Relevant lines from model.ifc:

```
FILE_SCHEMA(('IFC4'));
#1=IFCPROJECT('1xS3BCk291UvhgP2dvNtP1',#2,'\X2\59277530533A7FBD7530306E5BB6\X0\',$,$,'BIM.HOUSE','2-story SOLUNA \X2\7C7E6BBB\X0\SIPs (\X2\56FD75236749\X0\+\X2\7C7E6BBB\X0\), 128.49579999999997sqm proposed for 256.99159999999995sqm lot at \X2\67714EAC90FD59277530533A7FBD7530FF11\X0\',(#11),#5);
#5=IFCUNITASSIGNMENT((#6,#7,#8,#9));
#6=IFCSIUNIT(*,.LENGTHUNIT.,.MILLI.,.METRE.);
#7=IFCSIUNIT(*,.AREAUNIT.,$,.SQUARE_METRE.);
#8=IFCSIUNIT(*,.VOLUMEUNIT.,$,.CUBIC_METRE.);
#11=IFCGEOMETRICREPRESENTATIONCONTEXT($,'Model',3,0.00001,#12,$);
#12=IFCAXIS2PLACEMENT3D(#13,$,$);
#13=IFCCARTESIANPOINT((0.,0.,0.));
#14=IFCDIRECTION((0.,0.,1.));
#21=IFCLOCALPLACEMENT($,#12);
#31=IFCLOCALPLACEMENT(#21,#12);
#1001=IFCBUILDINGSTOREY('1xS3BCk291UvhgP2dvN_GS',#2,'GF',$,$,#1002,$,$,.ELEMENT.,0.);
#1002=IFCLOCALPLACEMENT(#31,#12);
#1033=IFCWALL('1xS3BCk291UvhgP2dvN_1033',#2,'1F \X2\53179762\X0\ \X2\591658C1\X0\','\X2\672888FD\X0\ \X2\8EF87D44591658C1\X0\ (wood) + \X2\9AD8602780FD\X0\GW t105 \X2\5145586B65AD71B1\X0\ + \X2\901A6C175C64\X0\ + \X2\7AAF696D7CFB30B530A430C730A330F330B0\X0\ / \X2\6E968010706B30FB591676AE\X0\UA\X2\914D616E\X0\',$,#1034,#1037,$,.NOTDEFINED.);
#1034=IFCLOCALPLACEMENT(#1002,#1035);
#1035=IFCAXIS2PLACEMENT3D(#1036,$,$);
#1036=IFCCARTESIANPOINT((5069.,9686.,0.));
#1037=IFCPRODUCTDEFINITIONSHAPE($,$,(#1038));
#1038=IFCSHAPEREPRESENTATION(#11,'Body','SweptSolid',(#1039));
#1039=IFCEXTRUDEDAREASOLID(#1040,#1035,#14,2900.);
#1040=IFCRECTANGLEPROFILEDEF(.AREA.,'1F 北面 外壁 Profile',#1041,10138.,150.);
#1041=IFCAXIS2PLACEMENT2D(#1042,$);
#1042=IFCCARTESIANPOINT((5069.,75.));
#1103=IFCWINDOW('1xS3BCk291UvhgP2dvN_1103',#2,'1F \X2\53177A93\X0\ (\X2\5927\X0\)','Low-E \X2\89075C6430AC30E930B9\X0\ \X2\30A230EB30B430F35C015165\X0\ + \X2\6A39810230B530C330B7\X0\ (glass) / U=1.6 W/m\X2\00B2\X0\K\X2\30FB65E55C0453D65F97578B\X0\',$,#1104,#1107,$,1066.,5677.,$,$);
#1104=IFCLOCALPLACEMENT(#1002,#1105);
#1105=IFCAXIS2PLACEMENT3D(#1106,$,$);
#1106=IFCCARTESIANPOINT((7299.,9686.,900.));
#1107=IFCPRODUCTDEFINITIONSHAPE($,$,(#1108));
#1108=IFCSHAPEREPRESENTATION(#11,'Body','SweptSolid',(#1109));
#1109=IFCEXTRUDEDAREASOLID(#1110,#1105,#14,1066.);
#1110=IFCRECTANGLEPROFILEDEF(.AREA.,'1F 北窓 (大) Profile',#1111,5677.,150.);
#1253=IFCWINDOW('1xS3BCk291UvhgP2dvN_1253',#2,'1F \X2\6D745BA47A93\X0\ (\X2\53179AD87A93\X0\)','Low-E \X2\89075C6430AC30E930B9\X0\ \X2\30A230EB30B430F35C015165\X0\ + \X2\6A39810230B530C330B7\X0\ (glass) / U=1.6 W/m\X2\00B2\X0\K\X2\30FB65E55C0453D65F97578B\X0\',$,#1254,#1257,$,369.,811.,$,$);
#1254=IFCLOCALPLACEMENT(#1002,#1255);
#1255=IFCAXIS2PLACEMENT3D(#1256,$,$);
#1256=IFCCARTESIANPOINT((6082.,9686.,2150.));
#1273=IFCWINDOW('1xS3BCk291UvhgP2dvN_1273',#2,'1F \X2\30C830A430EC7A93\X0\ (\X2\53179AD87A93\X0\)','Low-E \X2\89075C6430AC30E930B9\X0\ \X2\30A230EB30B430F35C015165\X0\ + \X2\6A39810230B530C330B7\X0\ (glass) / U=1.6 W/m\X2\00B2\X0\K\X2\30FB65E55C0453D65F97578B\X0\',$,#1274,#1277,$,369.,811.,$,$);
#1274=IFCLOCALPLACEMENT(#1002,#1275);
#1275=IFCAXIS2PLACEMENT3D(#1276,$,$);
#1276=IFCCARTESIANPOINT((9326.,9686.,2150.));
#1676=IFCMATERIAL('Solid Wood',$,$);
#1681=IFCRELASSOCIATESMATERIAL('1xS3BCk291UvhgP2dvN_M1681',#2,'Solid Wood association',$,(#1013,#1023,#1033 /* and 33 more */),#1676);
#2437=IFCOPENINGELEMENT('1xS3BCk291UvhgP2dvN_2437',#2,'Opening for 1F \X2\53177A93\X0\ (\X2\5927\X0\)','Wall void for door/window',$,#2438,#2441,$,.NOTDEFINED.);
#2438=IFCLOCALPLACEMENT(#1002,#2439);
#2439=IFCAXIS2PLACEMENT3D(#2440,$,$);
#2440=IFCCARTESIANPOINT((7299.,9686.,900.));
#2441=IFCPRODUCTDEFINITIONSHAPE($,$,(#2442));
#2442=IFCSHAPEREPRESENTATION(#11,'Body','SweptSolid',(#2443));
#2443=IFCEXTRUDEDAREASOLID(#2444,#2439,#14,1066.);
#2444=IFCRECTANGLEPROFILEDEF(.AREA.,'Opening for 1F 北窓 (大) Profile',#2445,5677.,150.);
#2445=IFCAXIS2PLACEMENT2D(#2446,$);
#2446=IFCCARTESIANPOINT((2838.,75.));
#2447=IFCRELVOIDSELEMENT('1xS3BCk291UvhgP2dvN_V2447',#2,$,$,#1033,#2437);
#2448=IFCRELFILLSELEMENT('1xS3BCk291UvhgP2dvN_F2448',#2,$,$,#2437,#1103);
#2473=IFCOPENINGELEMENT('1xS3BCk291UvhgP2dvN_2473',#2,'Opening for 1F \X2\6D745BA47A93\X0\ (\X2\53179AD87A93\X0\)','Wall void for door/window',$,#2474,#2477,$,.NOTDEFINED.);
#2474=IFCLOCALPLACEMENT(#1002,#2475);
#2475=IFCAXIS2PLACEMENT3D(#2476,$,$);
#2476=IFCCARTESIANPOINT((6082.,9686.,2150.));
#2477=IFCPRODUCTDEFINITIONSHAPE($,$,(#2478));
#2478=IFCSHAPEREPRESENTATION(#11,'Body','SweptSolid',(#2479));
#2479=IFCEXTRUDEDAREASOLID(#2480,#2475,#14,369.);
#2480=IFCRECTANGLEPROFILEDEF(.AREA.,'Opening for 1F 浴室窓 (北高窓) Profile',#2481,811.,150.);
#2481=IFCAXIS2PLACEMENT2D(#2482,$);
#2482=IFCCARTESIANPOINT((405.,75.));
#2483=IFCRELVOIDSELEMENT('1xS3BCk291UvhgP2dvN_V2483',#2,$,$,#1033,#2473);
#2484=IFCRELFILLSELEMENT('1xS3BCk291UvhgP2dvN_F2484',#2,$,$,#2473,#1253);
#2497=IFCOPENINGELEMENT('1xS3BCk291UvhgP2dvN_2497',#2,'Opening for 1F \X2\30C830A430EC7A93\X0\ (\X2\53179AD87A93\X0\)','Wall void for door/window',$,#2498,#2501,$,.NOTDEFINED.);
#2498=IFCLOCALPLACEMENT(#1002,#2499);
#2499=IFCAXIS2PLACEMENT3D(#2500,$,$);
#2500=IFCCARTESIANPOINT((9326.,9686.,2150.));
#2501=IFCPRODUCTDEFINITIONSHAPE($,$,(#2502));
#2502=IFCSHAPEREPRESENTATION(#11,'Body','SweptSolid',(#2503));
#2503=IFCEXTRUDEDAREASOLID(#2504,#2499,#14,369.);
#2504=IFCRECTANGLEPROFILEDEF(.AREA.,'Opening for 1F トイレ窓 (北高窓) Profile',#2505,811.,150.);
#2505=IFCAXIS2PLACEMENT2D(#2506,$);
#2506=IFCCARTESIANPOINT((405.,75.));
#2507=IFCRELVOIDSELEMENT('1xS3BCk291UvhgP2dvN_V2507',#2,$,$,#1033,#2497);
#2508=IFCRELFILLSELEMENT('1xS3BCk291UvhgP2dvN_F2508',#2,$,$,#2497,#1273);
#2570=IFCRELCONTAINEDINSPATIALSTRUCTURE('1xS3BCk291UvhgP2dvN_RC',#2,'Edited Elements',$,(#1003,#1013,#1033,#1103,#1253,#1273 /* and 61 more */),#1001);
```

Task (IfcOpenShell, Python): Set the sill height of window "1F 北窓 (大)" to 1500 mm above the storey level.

```python
import numpy as np
import ifcopenshell
import ifcopenshell.api.geometry
import ifcopenshell.geom
import ifcopenshell.util.element
import ifcopenshell.util.placement
import ifcopenshell.util.shape
import ifcopenshell.util.unit

model = ifcopenshell.open("model.ifc")
unit_scale = ifcopenshell.util.unit.calculate_unit_scale(model)

window = model.by_id(1103)
opening = window.FillsVoids[0].RelatingOpeningElement
storey = ifcopenshell.util.element.get_container(window, ifc_class="IfcBuildingStorey")
level = ifcopenshell.util.placement.get_local_placement(storey.ObjectPlacement)[2, 3]

# The opening's origin need not be at the sill, so measure its lowest point.
shape = ifcopenshell.geom.create_shape(ifcopenshell.geom.settings(), opening)
bottom = ifcopenshell.util.shape.get_shape_bottom_elevation(shape, shape.geometry) / unit_scale
dz = level + 1.5 / unit_scale - bottom

shift = np.array([0.0, 0.0, dz])
# The window is not placed relative to its opening, so move both.
for product in (opening, window):
    matrix = ifcopenshell.util.placement.get_local_placement(product.ObjectPlacement)
    matrix[:3, 3] += shift
    ifcopenshell.api.geometry.edit_object_placement(model, product=product, matrix=matrix, is_si=False)

print(f"moved by {dz * unit_scale:+.3f} m")

model.write("model_edited.ifc")
```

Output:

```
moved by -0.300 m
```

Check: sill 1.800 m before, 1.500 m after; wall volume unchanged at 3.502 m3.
